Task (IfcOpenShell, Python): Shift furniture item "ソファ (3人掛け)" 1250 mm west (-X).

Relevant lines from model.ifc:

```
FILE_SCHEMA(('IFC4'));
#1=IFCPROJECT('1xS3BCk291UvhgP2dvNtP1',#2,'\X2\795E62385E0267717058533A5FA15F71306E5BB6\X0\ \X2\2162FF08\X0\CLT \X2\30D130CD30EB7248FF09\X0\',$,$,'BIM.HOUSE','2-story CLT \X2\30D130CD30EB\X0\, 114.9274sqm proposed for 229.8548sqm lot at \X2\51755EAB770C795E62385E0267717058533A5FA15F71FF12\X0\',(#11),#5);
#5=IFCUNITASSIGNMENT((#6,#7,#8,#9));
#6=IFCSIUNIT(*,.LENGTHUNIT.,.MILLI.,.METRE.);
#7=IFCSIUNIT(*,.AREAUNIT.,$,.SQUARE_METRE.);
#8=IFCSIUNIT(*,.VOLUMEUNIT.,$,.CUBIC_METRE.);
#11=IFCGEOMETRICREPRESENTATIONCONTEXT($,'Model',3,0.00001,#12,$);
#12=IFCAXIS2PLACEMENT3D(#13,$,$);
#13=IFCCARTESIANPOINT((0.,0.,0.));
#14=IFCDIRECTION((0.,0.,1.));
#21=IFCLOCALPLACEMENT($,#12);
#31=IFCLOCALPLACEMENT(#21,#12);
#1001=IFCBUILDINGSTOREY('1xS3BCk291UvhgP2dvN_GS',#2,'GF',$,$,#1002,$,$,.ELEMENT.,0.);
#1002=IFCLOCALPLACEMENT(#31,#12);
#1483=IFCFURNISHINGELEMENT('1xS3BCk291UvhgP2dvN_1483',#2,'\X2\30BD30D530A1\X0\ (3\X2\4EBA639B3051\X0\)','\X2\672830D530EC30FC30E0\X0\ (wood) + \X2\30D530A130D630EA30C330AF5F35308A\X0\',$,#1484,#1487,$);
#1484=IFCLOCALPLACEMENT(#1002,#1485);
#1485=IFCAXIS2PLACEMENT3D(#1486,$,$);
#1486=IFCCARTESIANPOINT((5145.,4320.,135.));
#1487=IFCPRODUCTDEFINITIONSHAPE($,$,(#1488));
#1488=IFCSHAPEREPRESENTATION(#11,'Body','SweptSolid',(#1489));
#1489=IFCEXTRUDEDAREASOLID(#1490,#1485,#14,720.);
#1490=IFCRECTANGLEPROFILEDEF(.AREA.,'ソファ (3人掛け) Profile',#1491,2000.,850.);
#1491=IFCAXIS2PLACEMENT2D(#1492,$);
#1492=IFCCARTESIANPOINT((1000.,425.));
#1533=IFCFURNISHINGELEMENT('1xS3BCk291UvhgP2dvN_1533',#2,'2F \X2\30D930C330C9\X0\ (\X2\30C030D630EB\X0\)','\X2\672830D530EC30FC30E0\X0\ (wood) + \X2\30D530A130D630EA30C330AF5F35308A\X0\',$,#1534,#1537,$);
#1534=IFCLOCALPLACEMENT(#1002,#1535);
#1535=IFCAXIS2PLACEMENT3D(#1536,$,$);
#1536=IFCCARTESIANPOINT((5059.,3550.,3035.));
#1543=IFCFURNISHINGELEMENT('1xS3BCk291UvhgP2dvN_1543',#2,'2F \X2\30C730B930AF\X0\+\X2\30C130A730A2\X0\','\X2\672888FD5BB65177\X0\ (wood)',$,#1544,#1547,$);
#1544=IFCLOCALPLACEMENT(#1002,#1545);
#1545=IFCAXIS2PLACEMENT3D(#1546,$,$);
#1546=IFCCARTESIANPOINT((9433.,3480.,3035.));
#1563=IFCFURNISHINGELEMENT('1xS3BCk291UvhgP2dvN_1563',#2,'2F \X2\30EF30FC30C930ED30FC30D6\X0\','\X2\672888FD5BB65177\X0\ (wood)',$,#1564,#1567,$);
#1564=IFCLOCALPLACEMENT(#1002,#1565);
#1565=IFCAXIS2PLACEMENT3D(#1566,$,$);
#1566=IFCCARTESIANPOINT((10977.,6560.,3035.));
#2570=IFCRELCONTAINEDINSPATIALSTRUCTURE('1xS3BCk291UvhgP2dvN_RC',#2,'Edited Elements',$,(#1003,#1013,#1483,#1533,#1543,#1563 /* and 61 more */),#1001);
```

```python
import ifcopenshell
import ifcopenshell.api.geometry
import ifcopenshell.util.placement
import ifcopenshell.util.unit

model = ifcopenshell.open("model.ifc")
unit_scale = ifcopenshell.util.unit.calculate_unit_scale(model)

item = model.by_guid("1xS3BCk291UvhgP2dvN_1483")
matrix = ifcopenshell.util.placement.get_local_placement(item.ObjectPlacement)
matrix[0, 3] -= 1.25 / unit_scale
ifcopenshell.api.geometry.edit_object_placement(model, product=item, matrix=matrix, is_si=False)

print(ifcopenshell.util.placement.get_local_placement(item.ObjectPlacement).round(3) + 0.0)

model.write("model_rev.ifc")
```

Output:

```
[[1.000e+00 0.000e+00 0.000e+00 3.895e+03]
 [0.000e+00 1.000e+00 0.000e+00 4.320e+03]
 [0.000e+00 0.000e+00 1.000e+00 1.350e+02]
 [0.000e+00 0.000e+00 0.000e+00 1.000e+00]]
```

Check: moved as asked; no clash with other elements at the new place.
